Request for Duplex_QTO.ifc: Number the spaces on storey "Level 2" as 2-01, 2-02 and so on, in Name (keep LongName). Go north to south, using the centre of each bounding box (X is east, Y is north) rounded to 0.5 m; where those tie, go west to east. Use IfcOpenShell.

First a look at what the model holds.

```python
import ifcopenshell
import ifcopenshell.util.element
import ifcopenshell.util.placement

model = ifcopenshell.open("Duplex_QTO.ifc")
print(model.schema)
storey = next(s for s in model.by_type("IfcBuildingStorey") if s.Name == "Level 2")
spaces = [e for e in ifcopenshell.util.element.get_decomposition(storey) if e.is_a("IfcSpace")]
for e in sorted(spaces, key=lambda e: e.id()):
    origin = ifcopenshell.util.placement.get_local_placement(e.ObjectPlacement)[:3, 3]
    print(e.id(), e.Name, e.LongName, origin.round(2) + 0.0, sep=" | ")
```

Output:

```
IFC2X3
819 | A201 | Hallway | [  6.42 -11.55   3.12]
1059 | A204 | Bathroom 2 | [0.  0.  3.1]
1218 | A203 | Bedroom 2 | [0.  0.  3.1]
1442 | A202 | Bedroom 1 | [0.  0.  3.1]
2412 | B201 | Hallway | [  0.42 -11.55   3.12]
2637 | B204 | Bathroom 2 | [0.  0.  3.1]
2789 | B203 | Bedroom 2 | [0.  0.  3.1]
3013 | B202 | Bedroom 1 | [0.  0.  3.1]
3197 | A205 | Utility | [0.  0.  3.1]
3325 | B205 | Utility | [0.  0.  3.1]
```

```python
import ifcopenshell
import ifcopenshell.geom
import ifcopenshell.util.element
import ifcopenshell.util.shape

model = ifcopenshell.open("Duplex_QTO.ifc")
settings = ifcopenshell.geom.settings()
settings.set("use-world-coords", True)


def centre(element):
    shape = ifcopenshell.geom.create_shape(settings, element)
    return ifcopenshell.util.shape.get_bbox_centroid(shape.geometry)


storey = next(s for s in model.by_type("IfcBuildingStorey") if s.Name == "Level 2")
spaces = [e for e in ifcopenshell.util.element.get_decomposition(storey) if e.is_a("IfcSpace")]

# Insertion points can sit at a corner or the storey origin, so sort by the geometry (in metres).
centres = {e: centre(e) for e in spaces}
spaces.sort(key=lambda e: (-round(centres[e][1] / 0.5), centres[e][0]))

for i, e in enumerate(spaces, start=1):
    number = f"2-{i:02d}"
    e.Name = number
    print(e.id(), number)

model.write("Duplex_QTO-out.ifc")
```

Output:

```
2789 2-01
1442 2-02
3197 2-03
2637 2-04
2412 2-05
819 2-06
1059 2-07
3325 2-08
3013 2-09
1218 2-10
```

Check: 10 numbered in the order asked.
